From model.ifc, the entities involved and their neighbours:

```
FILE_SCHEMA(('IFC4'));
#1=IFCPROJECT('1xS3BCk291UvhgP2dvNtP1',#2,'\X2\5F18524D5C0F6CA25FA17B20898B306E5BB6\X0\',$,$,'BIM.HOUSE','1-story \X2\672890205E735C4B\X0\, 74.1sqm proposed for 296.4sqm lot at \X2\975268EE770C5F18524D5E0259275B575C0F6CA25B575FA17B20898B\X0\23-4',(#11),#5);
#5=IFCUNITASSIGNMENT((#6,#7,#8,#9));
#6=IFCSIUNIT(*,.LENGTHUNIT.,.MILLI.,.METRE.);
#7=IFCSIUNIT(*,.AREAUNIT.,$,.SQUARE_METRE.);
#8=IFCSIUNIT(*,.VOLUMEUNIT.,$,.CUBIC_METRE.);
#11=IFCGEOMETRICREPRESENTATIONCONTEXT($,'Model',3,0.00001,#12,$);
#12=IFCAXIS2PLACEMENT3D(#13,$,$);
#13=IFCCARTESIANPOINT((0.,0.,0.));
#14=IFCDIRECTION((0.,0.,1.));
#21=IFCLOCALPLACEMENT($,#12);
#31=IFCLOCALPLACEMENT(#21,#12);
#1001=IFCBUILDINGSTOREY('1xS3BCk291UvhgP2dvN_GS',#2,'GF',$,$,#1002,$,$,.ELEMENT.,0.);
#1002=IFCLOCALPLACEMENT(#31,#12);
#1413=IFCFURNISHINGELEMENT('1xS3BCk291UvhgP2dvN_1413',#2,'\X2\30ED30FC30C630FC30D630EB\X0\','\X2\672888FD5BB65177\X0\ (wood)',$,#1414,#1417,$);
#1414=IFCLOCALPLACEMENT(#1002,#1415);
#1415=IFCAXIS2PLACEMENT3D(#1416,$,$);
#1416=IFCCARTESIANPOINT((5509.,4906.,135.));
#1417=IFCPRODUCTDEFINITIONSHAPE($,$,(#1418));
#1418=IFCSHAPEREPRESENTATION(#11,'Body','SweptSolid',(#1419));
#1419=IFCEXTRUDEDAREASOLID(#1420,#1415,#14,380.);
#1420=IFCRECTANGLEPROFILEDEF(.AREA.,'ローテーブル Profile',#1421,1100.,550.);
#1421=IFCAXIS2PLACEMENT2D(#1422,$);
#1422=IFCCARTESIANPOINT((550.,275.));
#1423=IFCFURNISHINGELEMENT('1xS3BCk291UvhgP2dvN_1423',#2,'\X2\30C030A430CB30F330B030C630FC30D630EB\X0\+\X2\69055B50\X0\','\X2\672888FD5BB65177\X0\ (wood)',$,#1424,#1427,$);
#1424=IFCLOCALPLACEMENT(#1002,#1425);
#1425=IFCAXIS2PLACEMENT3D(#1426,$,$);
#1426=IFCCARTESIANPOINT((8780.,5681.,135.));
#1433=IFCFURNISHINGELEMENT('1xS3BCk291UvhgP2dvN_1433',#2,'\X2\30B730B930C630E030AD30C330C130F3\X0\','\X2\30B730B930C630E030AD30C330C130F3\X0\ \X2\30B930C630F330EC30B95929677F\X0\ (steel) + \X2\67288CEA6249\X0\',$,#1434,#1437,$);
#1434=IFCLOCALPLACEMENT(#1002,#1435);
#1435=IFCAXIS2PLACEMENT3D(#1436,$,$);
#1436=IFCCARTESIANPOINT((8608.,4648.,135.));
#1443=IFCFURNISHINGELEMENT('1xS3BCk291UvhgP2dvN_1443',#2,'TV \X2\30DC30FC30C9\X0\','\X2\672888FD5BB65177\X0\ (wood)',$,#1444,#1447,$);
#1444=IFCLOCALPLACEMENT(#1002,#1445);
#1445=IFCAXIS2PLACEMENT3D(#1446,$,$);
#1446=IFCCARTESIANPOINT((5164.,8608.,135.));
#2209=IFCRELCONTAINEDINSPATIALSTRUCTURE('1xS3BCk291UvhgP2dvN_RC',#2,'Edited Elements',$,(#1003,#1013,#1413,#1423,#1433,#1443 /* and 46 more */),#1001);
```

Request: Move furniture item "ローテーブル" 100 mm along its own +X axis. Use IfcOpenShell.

```python
import ifcopenshell
import ifcopenshell.api.geometry
import ifcopenshell.util.placement
import ifcopenshell.util.unit

model = ifcopenshell.open("model.ifc")
unit_scale = ifcopenshell.util.unit.calculate_unit_scale(model)

item = model.by_guid("1xS3BCk291UvhgP2dvN_1413")
matrix = ifcopenshell.util.placement.get_local_placement(item.ObjectPlacement)
matrix[:3, 3] += matrix[:3, 0] * 0.1 / unit_scale
ifcopenshell.api.geometry.edit_object_placement(model, product=item, matrix=matrix, is_si=False)

print(ifcopenshell.util.placement.get_local_placement(item.ObjectPlacement).round(3) + 0.0)

model.write("model_rev.ifc")
```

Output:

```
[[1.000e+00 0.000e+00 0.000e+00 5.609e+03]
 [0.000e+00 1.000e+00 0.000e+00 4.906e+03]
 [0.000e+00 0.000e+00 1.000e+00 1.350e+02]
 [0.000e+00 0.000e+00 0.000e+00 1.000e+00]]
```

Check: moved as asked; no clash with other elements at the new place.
